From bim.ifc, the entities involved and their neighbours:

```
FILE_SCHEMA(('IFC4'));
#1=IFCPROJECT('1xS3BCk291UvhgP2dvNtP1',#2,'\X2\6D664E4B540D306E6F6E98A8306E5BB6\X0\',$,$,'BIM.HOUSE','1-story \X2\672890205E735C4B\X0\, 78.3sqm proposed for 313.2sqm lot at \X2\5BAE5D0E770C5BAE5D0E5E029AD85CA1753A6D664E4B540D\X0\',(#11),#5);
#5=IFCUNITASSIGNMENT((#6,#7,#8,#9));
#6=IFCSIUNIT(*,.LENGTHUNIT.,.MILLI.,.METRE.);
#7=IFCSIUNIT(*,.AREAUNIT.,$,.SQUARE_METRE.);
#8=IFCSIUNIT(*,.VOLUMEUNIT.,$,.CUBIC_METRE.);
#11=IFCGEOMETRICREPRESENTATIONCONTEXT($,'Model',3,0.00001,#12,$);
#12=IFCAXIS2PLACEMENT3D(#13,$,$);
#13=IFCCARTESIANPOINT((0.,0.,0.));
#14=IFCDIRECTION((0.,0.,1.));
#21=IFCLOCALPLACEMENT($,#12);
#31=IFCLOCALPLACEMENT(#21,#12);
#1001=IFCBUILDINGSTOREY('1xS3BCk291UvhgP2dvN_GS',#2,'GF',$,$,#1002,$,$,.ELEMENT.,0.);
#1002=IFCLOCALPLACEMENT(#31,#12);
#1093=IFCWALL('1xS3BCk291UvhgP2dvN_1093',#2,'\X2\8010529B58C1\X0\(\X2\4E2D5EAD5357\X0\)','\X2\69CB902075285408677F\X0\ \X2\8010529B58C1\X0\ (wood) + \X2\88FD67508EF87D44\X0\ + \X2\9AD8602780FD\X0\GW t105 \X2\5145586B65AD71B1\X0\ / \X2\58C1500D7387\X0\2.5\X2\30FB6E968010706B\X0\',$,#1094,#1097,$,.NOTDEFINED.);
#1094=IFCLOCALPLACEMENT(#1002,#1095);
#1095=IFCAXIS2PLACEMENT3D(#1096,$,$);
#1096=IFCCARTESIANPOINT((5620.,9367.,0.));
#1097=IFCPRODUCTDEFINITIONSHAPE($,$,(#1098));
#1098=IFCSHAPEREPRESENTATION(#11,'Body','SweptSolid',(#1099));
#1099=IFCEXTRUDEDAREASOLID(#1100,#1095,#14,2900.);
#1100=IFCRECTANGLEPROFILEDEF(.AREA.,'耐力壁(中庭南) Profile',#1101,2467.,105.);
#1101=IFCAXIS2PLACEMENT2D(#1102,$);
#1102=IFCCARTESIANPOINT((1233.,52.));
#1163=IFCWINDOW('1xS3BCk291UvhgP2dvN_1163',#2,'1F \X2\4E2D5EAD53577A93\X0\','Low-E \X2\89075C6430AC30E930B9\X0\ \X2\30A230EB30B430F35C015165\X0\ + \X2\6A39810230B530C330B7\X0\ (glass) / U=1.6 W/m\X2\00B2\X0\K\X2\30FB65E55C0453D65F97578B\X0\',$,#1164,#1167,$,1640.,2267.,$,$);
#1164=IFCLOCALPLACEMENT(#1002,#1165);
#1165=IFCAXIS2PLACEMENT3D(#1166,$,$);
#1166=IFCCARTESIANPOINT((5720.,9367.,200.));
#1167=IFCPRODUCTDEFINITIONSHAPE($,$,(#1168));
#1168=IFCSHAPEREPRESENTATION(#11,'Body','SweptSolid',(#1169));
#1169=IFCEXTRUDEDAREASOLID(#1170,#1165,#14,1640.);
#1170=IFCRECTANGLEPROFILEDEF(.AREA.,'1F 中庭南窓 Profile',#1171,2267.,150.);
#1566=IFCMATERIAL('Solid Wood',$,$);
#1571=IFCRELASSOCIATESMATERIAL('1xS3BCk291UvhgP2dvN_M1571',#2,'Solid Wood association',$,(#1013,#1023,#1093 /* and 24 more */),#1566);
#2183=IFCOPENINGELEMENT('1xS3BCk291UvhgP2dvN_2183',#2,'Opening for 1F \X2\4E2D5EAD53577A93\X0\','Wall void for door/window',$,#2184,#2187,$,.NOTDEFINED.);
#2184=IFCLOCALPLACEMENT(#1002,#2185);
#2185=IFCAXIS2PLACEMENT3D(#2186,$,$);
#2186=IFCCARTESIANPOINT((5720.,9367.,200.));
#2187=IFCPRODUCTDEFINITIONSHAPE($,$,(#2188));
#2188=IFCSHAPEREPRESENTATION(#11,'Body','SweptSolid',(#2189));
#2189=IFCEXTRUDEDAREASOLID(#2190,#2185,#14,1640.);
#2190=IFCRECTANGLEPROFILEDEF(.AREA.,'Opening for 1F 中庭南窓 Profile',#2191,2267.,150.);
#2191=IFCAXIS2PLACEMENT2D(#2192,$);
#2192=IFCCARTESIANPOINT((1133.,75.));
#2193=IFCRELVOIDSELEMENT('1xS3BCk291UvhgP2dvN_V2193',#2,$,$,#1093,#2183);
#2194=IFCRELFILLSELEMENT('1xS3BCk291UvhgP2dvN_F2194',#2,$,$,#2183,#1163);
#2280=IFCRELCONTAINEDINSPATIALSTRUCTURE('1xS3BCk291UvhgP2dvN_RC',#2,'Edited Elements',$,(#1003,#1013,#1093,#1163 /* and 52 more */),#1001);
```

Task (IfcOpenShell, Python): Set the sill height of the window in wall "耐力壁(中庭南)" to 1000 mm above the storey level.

```python
import numpy as np
import ifcopenshell
import ifcopenshell.api.geometry
import ifcopenshell.geom
import ifcopenshell.util.element
import ifcopenshell.util.placement
import ifcopenshell.util.shape
import ifcopenshell.util.unit

model = ifcopenshell.open("bim.ifc")
unit_scale = ifcopenshell.util.unit.calculate_unit_scale(model)

window = model.by_guid("1xS3BCk291UvhgP2dvN_1163")
opening = window.FillsVoids[0].RelatingOpeningElement
storey = ifcopenshell.util.element.get_container(window, ifc_class="IfcBuildingStorey")
level = ifcopenshell.util.placement.get_local_placement(storey.ObjectPlacement)[2, 3]

# The opening's origin need not be at the sill, so measure its lowest point.
shape = ifcopenshell.geom.create_shape(ifcopenshell.geom.settings(), opening)
bottom = ifcopenshell.util.shape.get_shape_bottom_elevation(shape, shape.geometry) / unit_scale
dz = level + 1000.0 - bottom

shift = np.array([0.0, 0.0, dz])
# The window is not placed relative to its opening, so move both.
for product in (opening, window):
    matrix = ifcopenshell.util.placement.get_local_placement(product.ObjectPlacement)
    matrix[:3, 3] += shift
    ifcopenshell.api.geometry.edit_object_placement(model, product=product, matrix=matrix, is_si=False)

print(f"moved by {dz * unit_scale:+.3f} m")

model.write("bim-out.ifc")
```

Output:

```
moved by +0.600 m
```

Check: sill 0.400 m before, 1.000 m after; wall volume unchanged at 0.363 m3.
